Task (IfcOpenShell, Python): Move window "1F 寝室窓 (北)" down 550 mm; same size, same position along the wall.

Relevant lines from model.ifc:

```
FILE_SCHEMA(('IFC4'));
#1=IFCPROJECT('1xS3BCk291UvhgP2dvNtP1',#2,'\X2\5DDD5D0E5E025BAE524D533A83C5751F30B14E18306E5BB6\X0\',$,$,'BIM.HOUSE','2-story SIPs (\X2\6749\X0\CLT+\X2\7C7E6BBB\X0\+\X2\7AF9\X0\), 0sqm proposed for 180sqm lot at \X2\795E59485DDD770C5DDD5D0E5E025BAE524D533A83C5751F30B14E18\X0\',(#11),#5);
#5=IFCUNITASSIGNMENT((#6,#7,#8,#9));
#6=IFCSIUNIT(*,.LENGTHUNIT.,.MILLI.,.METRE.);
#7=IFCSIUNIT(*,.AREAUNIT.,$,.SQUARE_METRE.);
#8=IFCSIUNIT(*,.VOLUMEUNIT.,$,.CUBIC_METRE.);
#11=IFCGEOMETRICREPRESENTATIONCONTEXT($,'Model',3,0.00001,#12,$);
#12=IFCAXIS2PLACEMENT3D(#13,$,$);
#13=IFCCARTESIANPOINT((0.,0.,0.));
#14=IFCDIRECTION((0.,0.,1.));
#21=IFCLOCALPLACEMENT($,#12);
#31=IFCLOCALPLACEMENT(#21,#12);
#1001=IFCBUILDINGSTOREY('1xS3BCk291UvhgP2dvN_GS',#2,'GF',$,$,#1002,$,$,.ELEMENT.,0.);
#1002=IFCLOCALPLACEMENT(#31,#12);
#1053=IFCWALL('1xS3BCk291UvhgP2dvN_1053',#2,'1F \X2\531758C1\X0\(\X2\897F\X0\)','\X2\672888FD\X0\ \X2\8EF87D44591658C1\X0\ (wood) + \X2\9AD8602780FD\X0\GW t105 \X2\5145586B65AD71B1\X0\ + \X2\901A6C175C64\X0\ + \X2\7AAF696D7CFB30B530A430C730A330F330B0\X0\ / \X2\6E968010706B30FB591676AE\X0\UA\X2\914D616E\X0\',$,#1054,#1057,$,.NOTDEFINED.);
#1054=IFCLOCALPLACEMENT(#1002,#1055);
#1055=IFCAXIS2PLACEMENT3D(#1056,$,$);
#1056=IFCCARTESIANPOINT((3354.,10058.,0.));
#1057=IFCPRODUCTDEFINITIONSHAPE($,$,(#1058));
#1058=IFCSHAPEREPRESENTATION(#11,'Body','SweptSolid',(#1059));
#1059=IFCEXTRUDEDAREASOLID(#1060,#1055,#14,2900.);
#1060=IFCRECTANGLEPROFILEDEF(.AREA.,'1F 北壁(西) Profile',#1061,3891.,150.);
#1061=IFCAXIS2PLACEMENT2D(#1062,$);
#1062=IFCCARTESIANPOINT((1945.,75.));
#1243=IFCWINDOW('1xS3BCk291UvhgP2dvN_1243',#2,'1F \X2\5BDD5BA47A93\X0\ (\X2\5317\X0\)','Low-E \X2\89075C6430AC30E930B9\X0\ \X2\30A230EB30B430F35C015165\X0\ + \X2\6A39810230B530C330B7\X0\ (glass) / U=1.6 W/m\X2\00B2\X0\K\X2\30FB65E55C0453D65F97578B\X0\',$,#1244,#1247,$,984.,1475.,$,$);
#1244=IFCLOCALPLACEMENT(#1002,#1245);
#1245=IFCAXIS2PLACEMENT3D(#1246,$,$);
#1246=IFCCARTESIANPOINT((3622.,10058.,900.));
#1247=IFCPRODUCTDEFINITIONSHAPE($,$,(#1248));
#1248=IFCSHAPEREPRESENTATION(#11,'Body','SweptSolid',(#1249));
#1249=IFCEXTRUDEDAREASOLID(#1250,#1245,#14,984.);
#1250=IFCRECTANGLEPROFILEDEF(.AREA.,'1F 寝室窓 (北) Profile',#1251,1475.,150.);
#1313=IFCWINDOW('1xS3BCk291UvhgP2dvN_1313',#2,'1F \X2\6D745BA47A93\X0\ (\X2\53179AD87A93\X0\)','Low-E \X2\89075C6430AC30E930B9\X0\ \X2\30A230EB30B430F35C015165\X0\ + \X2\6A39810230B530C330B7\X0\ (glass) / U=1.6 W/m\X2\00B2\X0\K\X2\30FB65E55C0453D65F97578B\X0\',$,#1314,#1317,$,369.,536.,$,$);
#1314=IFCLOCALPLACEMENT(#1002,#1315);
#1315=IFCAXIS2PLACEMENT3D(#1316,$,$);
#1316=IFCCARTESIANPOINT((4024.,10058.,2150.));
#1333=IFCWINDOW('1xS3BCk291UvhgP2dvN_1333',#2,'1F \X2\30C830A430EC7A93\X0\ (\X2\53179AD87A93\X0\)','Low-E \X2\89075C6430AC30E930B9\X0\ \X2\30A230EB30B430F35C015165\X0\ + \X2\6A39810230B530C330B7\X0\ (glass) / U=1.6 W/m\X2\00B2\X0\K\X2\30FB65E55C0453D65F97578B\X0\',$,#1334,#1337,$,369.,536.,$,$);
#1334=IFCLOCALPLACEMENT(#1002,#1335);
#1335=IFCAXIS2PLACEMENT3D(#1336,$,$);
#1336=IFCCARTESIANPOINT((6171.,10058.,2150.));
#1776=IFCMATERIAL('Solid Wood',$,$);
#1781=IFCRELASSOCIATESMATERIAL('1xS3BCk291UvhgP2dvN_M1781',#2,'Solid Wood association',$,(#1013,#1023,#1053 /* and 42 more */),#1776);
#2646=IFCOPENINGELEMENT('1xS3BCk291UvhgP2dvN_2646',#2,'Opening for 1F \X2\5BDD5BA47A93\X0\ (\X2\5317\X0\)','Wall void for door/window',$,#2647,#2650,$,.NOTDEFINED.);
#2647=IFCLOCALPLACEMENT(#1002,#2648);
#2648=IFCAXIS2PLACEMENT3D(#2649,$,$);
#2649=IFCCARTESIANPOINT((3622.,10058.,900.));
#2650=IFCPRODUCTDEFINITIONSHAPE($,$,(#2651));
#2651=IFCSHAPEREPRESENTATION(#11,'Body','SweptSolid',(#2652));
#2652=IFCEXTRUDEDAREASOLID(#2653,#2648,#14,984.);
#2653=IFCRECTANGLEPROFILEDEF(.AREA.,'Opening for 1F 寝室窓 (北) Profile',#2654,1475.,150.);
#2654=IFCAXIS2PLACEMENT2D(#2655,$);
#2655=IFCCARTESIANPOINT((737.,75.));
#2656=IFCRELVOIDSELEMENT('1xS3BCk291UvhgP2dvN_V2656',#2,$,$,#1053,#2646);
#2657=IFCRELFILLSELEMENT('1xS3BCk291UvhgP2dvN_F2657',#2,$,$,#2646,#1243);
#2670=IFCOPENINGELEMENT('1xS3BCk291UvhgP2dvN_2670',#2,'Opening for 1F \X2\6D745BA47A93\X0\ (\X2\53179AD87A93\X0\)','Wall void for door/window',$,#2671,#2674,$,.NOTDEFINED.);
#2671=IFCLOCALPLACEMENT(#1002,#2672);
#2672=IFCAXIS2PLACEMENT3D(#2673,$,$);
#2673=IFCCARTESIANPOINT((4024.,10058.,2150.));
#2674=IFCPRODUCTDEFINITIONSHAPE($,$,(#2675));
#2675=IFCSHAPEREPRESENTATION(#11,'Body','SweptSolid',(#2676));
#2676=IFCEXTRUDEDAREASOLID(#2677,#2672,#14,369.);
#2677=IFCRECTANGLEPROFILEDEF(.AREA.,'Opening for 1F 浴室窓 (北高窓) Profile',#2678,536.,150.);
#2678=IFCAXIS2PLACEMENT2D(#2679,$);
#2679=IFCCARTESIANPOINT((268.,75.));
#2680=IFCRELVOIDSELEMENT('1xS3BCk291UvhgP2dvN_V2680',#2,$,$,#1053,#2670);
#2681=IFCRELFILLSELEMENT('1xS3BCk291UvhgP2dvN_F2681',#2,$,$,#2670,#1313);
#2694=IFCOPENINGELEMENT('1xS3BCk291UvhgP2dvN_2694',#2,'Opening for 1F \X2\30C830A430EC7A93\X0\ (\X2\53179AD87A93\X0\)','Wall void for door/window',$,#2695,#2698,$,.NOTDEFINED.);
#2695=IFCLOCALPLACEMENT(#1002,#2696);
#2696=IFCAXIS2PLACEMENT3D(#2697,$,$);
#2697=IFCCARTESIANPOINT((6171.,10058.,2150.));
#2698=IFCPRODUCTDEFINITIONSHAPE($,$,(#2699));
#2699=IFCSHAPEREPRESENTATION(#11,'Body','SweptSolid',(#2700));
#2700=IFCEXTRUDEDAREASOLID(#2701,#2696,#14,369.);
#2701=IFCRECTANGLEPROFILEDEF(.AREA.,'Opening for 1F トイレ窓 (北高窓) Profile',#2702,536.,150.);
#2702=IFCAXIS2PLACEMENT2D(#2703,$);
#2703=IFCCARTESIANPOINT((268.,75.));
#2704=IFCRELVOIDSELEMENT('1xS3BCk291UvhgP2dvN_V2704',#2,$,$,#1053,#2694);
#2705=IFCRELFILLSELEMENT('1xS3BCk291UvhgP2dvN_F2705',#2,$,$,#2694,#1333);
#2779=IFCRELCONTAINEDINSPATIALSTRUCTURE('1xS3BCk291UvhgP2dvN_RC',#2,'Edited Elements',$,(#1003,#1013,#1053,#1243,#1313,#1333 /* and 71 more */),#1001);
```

```python
import numpy as np
import ifcopenshell
import ifcopenshell.api.geometry
import ifcopenshell.util.placement
import ifcopenshell.util.unit

model = ifcopenshell.open("model.ifc")
unit_scale = ifcopenshell.util.unit.calculate_unit_scale(model)

window = model.by_guid("1xS3BCk291UvhgP2dvN_1243")
opening = window.FillsVoids[0].RelatingOpeningElement
dz = -0.55 / unit_scale

shift = np.array([0.0, 0.0, dz])
# The window is not placed relative to its opening, so move both.
for product in (opening, window):
    matrix = ifcopenshell.util.placement.get_local_placement(product.ObjectPlacement)
    matrix[:3, 3] += shift
    ifcopenshell.api.geometry.edit_object_placement(model, product=product, matrix=matrix, is_si=False)

print(f"moved by {dz * unit_scale:+.3f} m")

model.write("model_rev.ifc")
```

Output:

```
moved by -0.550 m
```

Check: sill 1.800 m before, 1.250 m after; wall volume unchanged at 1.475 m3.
